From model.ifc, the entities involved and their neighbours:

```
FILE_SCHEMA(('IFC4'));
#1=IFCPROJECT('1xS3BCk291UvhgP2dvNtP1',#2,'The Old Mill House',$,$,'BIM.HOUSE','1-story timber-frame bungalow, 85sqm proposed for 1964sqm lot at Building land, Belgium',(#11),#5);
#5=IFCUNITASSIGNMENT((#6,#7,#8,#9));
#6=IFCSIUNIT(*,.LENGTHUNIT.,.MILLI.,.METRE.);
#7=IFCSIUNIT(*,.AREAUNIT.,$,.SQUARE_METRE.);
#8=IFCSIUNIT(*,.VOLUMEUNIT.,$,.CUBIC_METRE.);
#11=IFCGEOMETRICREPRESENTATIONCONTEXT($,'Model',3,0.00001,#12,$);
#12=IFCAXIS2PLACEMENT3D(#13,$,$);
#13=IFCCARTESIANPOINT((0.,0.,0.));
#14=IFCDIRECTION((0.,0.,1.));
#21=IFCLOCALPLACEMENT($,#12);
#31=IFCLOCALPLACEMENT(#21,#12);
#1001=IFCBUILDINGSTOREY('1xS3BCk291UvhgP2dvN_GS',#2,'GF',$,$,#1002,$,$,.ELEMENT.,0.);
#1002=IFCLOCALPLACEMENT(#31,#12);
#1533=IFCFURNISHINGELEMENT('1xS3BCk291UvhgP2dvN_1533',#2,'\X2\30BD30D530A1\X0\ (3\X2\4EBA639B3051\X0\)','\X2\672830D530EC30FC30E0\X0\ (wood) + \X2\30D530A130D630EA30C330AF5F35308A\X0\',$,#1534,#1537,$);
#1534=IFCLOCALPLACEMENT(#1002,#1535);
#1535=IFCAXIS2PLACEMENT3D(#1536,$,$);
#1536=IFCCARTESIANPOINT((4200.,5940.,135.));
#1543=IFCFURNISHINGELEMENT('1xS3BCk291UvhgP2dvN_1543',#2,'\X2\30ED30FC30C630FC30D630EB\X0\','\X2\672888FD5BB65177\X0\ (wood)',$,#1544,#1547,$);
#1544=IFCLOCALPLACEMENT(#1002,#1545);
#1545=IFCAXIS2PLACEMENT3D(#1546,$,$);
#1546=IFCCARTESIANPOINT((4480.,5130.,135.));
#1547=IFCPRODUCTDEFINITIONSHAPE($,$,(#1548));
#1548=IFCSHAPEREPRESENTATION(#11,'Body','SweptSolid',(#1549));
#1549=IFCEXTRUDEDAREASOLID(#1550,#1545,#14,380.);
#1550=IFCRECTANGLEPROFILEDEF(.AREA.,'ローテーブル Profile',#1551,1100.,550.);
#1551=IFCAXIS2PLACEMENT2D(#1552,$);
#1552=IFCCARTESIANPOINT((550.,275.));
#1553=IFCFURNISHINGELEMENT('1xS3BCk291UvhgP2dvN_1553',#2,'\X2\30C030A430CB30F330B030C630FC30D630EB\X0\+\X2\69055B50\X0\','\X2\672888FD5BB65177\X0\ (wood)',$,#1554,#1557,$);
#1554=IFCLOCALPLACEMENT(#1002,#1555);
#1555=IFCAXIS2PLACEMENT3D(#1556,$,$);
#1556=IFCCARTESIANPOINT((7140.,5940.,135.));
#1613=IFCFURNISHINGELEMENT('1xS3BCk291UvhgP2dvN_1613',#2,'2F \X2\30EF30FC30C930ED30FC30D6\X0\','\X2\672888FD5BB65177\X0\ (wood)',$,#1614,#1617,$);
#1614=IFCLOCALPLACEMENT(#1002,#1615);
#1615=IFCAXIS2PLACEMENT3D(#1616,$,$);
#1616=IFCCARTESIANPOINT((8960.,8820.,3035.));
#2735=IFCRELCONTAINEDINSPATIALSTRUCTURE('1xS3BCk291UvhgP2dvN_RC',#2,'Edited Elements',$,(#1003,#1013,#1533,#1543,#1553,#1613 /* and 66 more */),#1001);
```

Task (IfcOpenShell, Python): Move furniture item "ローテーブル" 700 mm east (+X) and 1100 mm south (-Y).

```python
import ifcopenshell
import ifcopenshell.api.geometry
import ifcopenshell.util.placement

model = ifcopenshell.open("model.ifc")

item = model.by_id(1543)
matrix = ifcopenshell.util.placement.get_local_placement(item.ObjectPlacement)
matrix[0, 3] += 700.0
matrix[1, 3] -= 1100.0
ifcopenshell.api.geometry.edit_object_placement(model, product=item, matrix=matrix, is_si=False)

print(ifcopenshell.util.placement.get_local_placement(item.ObjectPlacement).round(3) + 0.0)

model.write("model_rev.ifc")
```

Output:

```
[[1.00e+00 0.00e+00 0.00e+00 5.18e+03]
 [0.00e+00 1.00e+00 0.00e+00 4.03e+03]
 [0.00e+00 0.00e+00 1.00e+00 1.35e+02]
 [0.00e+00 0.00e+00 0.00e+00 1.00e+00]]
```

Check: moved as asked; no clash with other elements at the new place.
